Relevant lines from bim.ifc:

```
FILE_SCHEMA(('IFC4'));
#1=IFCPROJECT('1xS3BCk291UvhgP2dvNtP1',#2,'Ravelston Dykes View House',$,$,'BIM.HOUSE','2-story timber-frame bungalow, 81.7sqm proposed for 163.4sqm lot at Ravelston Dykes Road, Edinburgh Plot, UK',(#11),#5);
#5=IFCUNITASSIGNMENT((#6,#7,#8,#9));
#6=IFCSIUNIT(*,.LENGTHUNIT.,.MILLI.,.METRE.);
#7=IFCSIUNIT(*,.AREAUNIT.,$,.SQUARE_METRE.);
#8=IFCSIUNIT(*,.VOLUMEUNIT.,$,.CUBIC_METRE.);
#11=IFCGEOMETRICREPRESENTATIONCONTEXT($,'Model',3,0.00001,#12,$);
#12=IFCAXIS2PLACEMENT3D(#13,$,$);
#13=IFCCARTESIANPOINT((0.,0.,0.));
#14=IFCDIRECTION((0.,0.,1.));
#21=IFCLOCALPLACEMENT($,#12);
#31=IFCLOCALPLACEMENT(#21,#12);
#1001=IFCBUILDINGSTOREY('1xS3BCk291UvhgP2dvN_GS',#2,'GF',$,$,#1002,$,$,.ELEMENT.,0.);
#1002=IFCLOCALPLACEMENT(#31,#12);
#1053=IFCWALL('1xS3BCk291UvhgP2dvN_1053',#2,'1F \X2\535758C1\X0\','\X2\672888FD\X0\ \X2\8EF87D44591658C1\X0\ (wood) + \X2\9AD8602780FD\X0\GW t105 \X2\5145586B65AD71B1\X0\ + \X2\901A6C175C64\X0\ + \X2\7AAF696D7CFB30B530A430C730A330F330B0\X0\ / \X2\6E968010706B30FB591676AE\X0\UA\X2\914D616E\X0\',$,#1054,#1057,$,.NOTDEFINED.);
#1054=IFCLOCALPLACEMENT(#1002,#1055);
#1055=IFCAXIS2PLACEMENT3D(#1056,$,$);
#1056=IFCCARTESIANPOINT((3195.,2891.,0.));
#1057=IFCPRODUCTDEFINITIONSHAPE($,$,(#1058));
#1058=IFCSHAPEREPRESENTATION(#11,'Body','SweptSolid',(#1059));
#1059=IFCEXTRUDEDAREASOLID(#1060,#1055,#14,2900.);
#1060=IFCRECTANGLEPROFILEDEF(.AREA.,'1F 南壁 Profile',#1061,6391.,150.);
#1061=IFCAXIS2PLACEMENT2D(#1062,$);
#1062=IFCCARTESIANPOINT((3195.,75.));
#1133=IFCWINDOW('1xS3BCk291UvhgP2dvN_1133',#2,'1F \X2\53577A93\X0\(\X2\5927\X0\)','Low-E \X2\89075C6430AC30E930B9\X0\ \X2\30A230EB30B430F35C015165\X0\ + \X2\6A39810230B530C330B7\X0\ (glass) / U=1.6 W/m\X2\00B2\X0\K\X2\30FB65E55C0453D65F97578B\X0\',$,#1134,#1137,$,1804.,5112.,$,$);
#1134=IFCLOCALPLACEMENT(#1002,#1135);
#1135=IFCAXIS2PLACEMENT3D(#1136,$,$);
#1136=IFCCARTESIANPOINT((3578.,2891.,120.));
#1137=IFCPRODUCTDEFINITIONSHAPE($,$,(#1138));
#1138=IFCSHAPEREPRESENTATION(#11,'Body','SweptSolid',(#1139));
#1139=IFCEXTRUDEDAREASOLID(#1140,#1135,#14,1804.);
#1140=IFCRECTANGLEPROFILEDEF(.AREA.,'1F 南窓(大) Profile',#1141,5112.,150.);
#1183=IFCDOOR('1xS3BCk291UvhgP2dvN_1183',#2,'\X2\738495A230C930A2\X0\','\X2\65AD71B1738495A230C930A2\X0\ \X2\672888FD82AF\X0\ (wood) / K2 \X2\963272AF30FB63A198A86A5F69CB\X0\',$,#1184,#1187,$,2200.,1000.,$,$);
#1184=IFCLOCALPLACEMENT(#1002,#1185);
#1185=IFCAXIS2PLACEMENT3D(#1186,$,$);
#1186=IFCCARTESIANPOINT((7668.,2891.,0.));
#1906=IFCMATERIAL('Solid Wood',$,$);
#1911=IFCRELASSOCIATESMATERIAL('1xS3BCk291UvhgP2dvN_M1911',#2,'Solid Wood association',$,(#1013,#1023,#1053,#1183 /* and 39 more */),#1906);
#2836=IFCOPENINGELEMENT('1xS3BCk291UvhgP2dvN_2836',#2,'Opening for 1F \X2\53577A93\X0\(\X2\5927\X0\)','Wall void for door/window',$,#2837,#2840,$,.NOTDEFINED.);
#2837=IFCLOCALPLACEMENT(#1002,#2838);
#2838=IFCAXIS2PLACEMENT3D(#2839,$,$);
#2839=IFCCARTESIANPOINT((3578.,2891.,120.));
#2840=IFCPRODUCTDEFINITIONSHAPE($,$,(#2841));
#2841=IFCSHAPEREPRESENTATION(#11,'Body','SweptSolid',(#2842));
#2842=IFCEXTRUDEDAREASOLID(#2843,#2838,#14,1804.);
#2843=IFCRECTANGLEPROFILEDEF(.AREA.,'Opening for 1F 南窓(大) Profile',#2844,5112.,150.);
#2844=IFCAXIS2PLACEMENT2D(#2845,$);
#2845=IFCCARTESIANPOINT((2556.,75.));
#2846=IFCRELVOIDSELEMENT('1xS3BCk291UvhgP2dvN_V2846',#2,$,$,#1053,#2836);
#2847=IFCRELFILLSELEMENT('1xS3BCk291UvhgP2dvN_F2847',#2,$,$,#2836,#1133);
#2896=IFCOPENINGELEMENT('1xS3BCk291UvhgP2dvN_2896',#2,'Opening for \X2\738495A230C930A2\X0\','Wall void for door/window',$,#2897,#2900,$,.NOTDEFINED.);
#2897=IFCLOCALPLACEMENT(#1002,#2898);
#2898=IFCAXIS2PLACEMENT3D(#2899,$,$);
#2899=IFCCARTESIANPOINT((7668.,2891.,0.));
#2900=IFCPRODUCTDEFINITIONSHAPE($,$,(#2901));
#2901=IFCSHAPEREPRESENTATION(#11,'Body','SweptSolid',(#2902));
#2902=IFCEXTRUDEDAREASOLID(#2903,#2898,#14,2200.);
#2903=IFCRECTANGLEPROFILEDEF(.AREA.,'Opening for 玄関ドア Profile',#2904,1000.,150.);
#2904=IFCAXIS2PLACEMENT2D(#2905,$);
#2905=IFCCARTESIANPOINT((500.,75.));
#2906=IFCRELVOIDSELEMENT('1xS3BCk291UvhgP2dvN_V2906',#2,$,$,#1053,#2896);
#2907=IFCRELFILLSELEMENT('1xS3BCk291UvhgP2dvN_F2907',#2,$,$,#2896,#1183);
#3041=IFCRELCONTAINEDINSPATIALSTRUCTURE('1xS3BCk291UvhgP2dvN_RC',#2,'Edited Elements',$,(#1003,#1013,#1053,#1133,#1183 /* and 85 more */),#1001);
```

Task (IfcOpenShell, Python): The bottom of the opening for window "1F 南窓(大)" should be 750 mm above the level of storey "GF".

```python
import numpy as np
import ifcopenshell
import ifcopenshell.api.geometry
import ifcopenshell.geom
import ifcopenshell.util.element
import ifcopenshell.util.placement
import ifcopenshell.util.shape
import ifcopenshell.util.unit

model = ifcopenshell.open("bim.ifc")
unit_scale = ifcopenshell.util.unit.calculate_unit_scale(model)

window = model.by_guid("1xS3BCk291UvhgP2dvN_1133")
opening = window.FillsVoids[0].RelatingOpeningElement
storey = ifcopenshell.util.element.get_container(window, ifc_class="IfcBuildingStorey")
level = ifcopenshell.util.placement.get_local_placement(storey.ObjectPlacement)[2, 3]

# The opening's origin need not be at the sill, so measure its lowest point.
shape = ifcopenshell.geom.create_shape(ifcopenshell.geom.settings(), opening)
bottom = ifcopenshell.util.shape.get_shape_bottom_elevation(shape, shape.geometry) / unit_scale
dz = level + 750.0 - bottom

shift = np.array([0.0, 0.0, dz])
# The window is not placed relative to its opening, so move both.
for product in (opening, window):
    matrix = ifcopenshell.util.placement.get_local_placement(product.ObjectPlacement)
    matrix[:3, 3] += shift
    ifcopenshell.api.geometry.edit_object_placement(model, product=product, matrix=matrix, is_si=False)

print(f"moved by {dz * unit_scale:+.3f} m")

model.write("bim_edited.ifc")
```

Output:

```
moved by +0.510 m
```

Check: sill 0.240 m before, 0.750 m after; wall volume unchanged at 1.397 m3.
